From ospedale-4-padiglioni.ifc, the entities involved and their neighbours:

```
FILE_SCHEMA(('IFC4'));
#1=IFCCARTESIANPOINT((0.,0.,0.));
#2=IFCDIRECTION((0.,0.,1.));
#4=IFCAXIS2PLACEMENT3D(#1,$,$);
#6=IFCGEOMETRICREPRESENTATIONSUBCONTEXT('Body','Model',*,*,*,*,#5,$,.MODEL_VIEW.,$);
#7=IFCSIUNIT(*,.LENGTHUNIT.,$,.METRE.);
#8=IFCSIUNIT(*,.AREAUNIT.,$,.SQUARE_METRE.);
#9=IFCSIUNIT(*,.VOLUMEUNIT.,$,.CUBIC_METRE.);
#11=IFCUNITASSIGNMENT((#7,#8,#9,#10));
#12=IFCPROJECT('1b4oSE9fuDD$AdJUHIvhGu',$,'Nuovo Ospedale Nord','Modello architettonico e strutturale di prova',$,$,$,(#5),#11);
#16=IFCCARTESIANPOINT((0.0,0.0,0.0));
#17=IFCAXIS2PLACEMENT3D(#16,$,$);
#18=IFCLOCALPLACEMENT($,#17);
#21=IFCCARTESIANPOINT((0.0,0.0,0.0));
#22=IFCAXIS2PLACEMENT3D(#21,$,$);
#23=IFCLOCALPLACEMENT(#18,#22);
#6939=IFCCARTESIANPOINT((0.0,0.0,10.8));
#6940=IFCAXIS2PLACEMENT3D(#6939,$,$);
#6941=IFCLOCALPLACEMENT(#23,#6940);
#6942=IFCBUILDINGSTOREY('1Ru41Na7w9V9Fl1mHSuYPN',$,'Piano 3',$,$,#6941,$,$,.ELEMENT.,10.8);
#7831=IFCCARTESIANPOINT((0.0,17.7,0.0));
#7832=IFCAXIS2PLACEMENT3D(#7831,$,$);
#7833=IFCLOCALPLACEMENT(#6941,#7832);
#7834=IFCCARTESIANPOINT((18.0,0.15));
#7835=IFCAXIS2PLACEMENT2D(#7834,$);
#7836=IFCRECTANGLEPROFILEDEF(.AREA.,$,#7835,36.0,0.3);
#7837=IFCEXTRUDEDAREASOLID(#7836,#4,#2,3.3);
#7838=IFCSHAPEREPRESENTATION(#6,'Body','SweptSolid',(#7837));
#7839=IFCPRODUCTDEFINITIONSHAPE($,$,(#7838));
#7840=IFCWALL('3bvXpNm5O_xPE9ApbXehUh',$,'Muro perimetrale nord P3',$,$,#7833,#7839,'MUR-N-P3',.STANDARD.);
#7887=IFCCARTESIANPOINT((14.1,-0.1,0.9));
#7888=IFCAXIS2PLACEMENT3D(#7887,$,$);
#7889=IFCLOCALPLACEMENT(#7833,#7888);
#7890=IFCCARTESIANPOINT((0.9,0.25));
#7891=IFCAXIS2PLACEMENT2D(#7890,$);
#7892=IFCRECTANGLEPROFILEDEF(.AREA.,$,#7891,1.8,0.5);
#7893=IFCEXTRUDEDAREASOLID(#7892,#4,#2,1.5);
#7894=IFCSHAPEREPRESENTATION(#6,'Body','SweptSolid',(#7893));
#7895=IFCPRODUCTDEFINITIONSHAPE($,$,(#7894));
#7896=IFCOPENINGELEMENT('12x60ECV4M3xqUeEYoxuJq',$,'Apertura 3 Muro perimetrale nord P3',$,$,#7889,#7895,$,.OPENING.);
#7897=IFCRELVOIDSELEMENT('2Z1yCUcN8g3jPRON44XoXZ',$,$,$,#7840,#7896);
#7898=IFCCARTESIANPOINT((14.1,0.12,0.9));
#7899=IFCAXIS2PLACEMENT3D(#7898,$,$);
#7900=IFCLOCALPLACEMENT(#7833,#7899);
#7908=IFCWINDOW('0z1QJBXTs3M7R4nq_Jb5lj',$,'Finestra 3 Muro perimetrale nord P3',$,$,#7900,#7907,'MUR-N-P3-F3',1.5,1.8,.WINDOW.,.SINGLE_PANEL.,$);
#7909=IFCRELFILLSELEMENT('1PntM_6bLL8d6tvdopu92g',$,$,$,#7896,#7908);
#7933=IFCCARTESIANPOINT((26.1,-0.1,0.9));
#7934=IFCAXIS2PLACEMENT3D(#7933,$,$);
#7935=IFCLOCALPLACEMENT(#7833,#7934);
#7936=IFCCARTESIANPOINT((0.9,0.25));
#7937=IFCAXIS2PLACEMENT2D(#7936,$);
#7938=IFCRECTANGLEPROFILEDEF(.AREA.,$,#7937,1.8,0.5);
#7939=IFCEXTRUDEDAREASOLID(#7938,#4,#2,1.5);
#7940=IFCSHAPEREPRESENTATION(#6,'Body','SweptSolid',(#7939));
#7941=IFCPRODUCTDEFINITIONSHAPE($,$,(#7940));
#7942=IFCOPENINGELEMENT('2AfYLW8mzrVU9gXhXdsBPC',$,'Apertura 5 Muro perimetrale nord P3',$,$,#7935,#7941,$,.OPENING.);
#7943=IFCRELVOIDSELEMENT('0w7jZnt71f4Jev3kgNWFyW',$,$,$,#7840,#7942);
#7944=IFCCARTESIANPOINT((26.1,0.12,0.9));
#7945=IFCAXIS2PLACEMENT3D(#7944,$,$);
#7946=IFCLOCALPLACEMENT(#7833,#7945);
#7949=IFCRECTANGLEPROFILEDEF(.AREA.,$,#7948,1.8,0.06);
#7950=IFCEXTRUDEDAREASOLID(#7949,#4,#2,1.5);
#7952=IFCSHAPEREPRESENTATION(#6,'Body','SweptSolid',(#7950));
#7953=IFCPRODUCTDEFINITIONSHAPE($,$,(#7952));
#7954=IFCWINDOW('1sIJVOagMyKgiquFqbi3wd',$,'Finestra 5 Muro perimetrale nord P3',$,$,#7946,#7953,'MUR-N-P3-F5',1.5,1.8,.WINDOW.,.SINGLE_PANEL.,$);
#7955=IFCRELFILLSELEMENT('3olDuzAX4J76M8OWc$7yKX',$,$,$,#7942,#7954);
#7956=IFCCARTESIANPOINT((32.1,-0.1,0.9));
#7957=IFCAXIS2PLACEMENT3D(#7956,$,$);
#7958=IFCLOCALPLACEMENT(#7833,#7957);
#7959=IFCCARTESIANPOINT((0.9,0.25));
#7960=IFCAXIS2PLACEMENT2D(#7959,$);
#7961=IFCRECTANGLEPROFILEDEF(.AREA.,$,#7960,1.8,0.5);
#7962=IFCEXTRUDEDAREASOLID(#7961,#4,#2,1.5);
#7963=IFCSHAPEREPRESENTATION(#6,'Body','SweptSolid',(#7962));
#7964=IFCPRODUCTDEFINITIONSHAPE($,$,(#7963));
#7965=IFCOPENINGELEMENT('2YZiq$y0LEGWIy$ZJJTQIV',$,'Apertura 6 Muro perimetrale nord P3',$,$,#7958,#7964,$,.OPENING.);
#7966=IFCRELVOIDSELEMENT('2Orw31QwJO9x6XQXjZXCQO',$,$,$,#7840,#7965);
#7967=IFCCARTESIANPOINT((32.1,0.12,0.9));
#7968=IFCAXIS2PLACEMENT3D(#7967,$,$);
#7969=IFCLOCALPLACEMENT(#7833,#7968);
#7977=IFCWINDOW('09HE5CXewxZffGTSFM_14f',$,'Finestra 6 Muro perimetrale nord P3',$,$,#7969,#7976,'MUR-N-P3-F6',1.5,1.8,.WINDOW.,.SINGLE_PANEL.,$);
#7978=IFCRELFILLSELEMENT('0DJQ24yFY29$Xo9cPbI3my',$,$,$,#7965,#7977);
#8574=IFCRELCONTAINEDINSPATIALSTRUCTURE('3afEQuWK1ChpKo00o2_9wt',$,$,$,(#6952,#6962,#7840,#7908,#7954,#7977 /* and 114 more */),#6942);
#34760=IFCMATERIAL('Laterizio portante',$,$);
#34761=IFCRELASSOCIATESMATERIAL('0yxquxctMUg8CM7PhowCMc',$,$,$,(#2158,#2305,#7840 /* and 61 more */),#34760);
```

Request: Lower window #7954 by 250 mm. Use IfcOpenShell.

```python
import numpy as np
import ifcopenshell
import ifcopenshell.api.geometry
import ifcopenshell.util.placement
import ifcopenshell.util.unit

model = ifcopenshell.open("ospedale-4-padiglioni.ifc")
unit_scale = ifcopenshell.util.unit.calculate_unit_scale(model)

window = model.by_guid("1sIJVOagMyKgiquFqbi3wd")
opening = window.FillsVoids[0].RelatingOpeningElement
dz = -0.25 / unit_scale

shift = np.array([0.0, 0.0, dz])
# The window is not placed relative to its opening, so move both.
for product in (opening, window):
    matrix = ifcopenshell.util.placement.get_local_placement(product.ObjectPlacement)
    matrix[:3, 3] += shift
    ifcopenshell.api.geometry.edit_object_placement(model, product=product, matrix=matrix, is_si=False)

print(f"moved by {dz * unit_scale:+.3f} m")

model.write("ospedale-4-padiglioni-out.ifc")
```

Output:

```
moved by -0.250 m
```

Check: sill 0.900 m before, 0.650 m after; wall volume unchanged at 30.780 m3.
